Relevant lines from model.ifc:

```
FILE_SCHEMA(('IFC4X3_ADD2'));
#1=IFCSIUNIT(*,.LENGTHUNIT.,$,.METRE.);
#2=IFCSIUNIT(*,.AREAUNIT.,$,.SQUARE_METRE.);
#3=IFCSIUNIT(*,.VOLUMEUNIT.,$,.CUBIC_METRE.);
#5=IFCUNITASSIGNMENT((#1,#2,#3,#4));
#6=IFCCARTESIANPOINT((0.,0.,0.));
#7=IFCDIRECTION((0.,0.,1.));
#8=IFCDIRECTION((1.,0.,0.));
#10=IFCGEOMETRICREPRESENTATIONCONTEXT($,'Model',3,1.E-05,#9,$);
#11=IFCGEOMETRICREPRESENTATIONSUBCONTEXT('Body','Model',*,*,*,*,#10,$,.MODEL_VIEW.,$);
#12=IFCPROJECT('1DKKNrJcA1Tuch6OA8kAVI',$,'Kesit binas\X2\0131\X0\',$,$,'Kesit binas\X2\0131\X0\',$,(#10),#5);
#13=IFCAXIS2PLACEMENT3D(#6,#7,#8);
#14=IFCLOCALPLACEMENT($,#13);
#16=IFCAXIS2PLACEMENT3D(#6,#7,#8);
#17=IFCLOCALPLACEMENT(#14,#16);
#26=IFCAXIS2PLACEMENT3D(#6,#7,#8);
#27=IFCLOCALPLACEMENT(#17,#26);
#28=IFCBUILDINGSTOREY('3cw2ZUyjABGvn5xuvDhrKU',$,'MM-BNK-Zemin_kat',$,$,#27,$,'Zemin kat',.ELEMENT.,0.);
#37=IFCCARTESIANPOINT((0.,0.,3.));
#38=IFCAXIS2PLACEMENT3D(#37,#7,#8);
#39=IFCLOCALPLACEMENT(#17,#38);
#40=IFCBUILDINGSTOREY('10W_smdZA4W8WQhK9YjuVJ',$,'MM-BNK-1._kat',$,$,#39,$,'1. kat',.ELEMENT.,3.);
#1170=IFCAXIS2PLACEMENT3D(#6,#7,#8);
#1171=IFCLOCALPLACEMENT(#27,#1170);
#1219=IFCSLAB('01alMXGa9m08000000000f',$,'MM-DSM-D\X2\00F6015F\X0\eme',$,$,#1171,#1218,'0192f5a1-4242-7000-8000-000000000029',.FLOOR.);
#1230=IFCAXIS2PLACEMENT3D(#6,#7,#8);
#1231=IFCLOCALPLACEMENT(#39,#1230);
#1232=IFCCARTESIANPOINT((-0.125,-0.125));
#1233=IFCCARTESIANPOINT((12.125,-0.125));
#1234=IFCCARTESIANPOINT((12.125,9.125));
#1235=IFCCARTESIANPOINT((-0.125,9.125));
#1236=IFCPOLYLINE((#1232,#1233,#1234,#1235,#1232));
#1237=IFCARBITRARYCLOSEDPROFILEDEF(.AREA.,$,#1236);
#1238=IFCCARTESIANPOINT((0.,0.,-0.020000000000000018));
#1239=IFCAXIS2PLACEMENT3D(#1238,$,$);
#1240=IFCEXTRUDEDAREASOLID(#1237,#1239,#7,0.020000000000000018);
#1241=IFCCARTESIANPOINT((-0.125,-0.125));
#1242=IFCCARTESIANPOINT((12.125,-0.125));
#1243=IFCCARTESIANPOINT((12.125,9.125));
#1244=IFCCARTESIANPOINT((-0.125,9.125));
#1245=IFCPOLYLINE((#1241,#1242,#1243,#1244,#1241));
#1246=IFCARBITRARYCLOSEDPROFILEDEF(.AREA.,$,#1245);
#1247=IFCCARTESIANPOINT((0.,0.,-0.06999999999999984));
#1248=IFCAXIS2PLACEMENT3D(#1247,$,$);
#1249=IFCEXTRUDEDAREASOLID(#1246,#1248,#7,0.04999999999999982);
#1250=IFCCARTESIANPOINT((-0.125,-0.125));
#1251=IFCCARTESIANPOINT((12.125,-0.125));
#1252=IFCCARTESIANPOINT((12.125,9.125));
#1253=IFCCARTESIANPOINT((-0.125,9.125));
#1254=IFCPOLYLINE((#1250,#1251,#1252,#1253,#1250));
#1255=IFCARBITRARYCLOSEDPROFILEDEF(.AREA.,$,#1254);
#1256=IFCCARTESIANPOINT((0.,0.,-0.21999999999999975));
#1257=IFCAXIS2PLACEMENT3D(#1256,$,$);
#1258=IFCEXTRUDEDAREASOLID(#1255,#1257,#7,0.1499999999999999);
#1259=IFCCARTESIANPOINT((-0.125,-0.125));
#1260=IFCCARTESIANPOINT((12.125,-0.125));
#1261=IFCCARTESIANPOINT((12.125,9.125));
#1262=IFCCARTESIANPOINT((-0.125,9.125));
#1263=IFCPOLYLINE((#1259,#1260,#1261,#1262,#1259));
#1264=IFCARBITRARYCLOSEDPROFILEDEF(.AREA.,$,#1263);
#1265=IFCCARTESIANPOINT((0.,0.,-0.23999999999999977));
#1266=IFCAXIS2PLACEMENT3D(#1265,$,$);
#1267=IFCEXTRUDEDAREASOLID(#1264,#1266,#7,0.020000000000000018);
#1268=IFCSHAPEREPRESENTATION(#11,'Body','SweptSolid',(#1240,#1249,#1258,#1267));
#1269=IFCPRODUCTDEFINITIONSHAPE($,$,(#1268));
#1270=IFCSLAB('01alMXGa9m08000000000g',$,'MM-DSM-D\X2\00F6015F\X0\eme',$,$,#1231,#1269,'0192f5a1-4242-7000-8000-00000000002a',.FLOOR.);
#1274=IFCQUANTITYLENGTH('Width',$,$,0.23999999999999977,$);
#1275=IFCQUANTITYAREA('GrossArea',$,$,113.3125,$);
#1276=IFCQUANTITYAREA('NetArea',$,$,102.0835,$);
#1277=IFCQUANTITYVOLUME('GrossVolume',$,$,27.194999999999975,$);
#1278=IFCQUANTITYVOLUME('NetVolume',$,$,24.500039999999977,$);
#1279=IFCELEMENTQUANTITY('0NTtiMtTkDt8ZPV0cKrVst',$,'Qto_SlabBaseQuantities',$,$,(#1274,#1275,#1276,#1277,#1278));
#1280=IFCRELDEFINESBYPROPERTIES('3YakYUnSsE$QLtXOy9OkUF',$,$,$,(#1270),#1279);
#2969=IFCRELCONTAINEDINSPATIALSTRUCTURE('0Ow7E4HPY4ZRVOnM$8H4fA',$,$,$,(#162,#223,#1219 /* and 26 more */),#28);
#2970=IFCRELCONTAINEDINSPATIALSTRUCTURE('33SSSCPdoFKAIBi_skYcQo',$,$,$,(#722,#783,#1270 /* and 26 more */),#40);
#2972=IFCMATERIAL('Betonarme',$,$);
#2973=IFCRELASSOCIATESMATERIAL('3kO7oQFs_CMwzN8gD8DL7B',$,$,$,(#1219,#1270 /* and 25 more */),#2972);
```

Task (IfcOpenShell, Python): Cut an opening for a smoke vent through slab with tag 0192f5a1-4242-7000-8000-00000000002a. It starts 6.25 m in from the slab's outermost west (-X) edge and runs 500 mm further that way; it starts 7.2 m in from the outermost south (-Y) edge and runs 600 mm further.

```python
import numpy as np
import ifcopenshell
import ifcopenshell.api.feature
import ifcopenshell.api.geometry
import ifcopenshell.api.pset
import ifcopenshell.api.root
import ifcopenshell.geom
import ifcopenshell.util.element
import ifcopenshell.util.placement
import ifcopenshell.util.representation
import ifcopenshell.util.shape
import ifcopenshell.util.unit

model = ifcopenshell.open("model.ifc")
unit_scale = ifcopenshell.util.unit.calculate_unit_scale(model)
area_scale = ifcopenshell.util.unit.calculate_unit_scale(model, "AREAUNIT")
volume_scale = ifcopenshell.util.unit.calculate_unit_scale(model, "VOLUMEUNIT")
settings = ifcopenshell.geom.settings()


def volume(element):
    """Net volume in cubic metres, openings subtracted."""
    shape = ifcopenshell.geom.create_shape(settings, element)
    return ifcopenshell.util.shape.get_volume(shape.geometry)


slab = model.by_guid("01alMXGa9m08000000000g")
before = volume(slab)

# Extent in the slab's own axes, in metres. The edges named are its -X and -Y sides.
slab_shape = ifcopenshell.geom.create_shape(settings, slab)
vertices = ifcopenshell.util.shape.get_vertices(slab_shape.geometry)
x_min, y_min, bottom = vertices.min(axis=0)
top = vertices[:, 2].max()

opening = ifcopenshell.api.root.create_entity(model, ifc_class="IfcOpeningElement", name="Smoke vent opening", predefined_type="OPENING")
context = ifcopenshell.util.representation.get_context(model, "Model", "Body", "MODEL_VIEW")
width, depth = 0.5, 0.6
outline = [(0.0, 0.0), (width, 0.0), (width, depth), (0.0, depth), (0.0, 0.0)]
# Overshoot both faces by 50 mm so the cut is clean.
shape = ifcopenshell.api.geometry.add_slab_representation(
    model, context=context, depth=top - bottom + 0.1, polyline=outline
)
ifcopenshell.api.geometry.assign_representation(model, product=opening, representation=shape)

matrix = ifcopenshell.util.placement.get_local_placement(slab.ObjectPlacement)
matrix[:, 3] = matrix @ np.append(np.array([x_min + 6.25, y_min + 7.2, bottom - 0.05]) / unit_scale, 1.0)
ifcopenshell.api.geometry.edit_object_placement(model, product=opening, matrix=matrix, is_si=False)
ifcopenshell.api.feature.add_feature(model, feature=opening, element=slab)

after = volume(slab)

# Update the slab's stored quantities.
qto = model.by_id(ifcopenshell.util.element.get_pset(slab, "Qto_SlabBaseQuantities", should_inherit=False)["id"])
ifcopenshell.api.pset.edit_qto(model, qto=qto, properties={
    "NetArea": after / (top - bottom) / area_scale,
    "NetVolume": after / volume_scale,
})

print(f"slab volume {before:.3f} -> {after:.3f} m3")

model.write("model-out.ifc")
```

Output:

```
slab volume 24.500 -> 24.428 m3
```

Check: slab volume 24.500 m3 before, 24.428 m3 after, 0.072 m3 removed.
